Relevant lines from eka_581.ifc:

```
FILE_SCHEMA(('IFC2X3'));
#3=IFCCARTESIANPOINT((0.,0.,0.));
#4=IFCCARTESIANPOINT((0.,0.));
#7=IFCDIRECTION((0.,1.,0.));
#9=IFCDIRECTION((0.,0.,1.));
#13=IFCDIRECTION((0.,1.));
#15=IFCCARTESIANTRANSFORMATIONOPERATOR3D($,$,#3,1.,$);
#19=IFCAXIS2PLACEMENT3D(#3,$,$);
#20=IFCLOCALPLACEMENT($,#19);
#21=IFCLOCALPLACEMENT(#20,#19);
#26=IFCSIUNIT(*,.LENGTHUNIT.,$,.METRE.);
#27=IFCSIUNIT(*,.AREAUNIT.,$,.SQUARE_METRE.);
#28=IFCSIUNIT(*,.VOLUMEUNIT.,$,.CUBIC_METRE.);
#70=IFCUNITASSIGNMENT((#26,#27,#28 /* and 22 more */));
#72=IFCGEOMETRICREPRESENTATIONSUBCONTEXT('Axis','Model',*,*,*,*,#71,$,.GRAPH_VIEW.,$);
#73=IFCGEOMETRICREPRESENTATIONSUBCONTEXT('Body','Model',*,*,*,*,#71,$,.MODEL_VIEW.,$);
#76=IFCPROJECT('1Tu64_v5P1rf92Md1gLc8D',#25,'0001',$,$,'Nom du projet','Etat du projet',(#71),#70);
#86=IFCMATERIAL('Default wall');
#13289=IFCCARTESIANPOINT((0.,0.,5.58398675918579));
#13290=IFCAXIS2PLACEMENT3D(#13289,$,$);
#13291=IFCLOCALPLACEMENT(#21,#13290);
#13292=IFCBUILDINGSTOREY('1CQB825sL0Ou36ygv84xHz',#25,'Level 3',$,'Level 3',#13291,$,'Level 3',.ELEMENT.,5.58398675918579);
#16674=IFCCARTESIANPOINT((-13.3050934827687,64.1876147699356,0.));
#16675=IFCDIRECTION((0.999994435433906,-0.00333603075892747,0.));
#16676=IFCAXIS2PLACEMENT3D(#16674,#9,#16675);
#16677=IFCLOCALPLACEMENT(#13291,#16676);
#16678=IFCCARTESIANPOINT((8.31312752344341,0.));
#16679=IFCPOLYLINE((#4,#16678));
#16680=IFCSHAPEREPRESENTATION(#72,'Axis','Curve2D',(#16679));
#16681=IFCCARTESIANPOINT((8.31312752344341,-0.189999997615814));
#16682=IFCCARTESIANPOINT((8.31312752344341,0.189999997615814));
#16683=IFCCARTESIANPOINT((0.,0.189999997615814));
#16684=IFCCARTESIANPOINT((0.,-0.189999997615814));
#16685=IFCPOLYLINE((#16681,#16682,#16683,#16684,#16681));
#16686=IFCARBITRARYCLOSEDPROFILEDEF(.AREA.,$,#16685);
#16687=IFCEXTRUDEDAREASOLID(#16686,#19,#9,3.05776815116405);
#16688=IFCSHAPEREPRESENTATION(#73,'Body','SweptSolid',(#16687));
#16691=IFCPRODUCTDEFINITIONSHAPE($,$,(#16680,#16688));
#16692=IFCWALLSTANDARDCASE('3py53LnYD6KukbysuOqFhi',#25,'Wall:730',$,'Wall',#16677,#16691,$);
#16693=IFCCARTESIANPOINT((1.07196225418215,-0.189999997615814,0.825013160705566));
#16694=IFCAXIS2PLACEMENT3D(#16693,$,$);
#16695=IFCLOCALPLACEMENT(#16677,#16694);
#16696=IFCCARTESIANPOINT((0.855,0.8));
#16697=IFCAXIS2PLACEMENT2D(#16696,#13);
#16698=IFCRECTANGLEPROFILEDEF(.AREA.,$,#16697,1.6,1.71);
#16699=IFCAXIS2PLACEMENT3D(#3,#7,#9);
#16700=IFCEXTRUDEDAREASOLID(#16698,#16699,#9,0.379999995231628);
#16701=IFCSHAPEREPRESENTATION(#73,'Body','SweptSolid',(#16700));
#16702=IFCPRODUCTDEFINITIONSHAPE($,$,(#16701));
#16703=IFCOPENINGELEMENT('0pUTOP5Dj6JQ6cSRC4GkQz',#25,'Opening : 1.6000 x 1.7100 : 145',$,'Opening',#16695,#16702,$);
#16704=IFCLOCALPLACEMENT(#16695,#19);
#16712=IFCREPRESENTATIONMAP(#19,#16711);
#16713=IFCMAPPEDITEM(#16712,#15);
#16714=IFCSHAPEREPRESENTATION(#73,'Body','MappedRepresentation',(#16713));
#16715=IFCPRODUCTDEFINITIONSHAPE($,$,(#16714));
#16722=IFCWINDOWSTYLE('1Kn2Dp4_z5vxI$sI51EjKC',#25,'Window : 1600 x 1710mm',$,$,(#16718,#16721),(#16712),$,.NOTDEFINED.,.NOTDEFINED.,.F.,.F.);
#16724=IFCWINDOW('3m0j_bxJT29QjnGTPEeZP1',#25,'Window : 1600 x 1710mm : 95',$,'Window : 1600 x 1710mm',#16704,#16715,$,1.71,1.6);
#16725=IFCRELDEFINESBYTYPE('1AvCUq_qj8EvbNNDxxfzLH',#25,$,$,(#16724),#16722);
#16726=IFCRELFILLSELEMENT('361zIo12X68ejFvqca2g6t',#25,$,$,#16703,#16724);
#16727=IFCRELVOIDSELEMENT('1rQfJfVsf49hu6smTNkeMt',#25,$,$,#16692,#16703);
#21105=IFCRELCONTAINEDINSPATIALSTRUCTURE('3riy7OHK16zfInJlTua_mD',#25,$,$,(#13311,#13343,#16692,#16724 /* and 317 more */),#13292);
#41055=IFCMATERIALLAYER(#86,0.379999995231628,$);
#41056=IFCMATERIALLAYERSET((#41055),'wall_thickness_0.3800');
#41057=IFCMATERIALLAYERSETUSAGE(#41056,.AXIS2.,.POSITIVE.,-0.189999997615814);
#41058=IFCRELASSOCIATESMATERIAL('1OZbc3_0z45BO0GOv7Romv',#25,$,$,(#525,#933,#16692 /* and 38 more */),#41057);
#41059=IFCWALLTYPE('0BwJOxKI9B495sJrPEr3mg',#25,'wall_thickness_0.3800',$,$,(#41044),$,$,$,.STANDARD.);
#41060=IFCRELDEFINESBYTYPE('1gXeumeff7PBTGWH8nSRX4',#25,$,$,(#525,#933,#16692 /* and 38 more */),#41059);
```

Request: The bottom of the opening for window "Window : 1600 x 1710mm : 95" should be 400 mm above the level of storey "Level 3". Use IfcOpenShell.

```python
import numpy as np
import ifcopenshell
import ifcopenshell.api.geometry
import ifcopenshell.geom
import ifcopenshell.util.element
import ifcopenshell.util.placement
import ifcopenshell.util.shape
import ifcopenshell.util.unit

model = ifcopenshell.open("eka_581.ifc")
unit_scale = ifcopenshell.util.unit.calculate_unit_scale(model)

window = model.by_guid("3m0j_bxJT29QjnGTPEeZP1")
opening = window.FillsVoids[0].RelatingOpeningElement
storey = ifcopenshell.util.element.get_container(window, ifc_class="IfcBuildingStorey")
level = ifcopenshell.util.placement.get_local_placement(storey.ObjectPlacement)[2, 3]

# The opening's origin need not be at the sill, so measure its lowest point.
shape = ifcopenshell.geom.create_shape(ifcopenshell.geom.settings(), opening)
bottom = ifcopenshell.util.shape.get_shape_bottom_elevation(shape, shape.geometry) / unit_scale
dz = level + 0.4 / unit_scale - bottom

shift = np.array([0.0, 0.0, dz])
# The window is placed relative to its opening, so it follows when the opening moves.
matrix = ifcopenshell.util.placement.get_local_placement(opening.ObjectPlacement)
matrix[:3, 3] += shift
ifcopenshell.api.geometry.edit_object_placement(
    model, product=opening, matrix=matrix, is_si=False, should_transform_children=True
)

print(f"moved by {dz * unit_scale:+.3f} m")

model.write("eka_581_rev.ifc")
```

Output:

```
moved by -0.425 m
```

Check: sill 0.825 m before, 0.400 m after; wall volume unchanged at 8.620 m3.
